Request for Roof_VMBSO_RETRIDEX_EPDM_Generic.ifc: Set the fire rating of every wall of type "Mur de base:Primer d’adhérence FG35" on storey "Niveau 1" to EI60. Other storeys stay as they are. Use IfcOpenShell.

First a look at what the model holds.

```python
import ifcopenshell
import ifcopenshell.util.element

model = ifcopenshell.open("Roof_VMBSO_RETRIDEX_EPDM_Generic.ifc")
print(model.schema)
storey = next(s for s in model.by_type("IfcBuildingStorey") if s.Name == "Niveau 1")
walls = [e for e in ifcopenshell.util.element.get_decomposition(storey) if e.is_a("IfcWall")]
seen = {}
for e in walls:
    element_type = ifcopenshell.util.element.get_type(e)
    key = (element_type.Name if element_type != e and element_type else None, ifcopenshell.util.element.get_pset(e, "Pset_WallCommon", "FireRating"))
    seen[key] = seen.get(key, 0) + 1
for (name, value), count in sorted(seen.items(), key=str):
    print(count, "x", name, "|", value)
```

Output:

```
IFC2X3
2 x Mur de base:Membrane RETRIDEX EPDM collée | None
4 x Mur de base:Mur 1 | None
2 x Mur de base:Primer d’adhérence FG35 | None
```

```python
import ifcopenshell
import ifcopenshell.api.pset
import ifcopenshell.util.element

model = ifcopenshell.open("Roof_VMBSO_RETRIDEX_EPDM_Generic.ifc")

storey = next(s for s in model.by_type("IfcBuildingStorey") if s.Name == "Niveau 1")
walls = [e for e in ifcopenshell.util.element.get_decomposition(storey) if e.is_a("IfcWall")]

count = 0
for e in walls:
    element_type = ifcopenshell.util.element.get_type(e)
    if element_type in (None, e) or element_type.Name != "Mur de base:Primer d’adhérence FG35":
        continue
    # add_pset returns the element's existing set when there is one.
    pset = ifcopenshell.api.pset.add_pset(model, product=e, name="Pset_WallCommon")
    ifcopenshell.api.pset.edit_pset(model, pset=pset, properties={"FireRating": "EI60"})
    count += 1

print(count, "walls updated")

model.write("Roof_VMBSO_RETRIDEX_EPDM_Generic-out.ifc")
```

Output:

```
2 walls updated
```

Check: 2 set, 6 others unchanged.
